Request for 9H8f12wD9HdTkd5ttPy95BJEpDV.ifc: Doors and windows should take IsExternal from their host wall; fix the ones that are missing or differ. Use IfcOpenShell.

First a look at what the model holds.

```python
import ifcopenshell
import ifcopenshell.util.element

model = ifcopenshell.open("9H8f12wD9HdTkd5ttPy95BJEpDV.ifc")
print(model.schema)
seen = {}
for e in model.by_type("IfcDoor") + model.by_type("IfcWindow"):
    if not e.FillsVoids:
        continue
    host = e.FillsVoids[0].RelatingOpeningElement.VoidsElements[0].RelatingBuildingElement
    own = ifcopenshell.util.element.get_pset(e, f"Pset_{e.is_a()[3:].removesuffix('StandardCase')}Common", "IsExternal")
    wall = ifcopenshell.util.element.get_pset(host, "Pset_WallCommon", "IsExternal")
    seen[e.is_a(), own, wall] = seen.get((e.is_a(), own, wall), 0) + 1
for (cls, own, wall), count in sorted(seen.items(), key=str):
    print(count, cls, "IsExternal:", own, "| host wall:", wall)
```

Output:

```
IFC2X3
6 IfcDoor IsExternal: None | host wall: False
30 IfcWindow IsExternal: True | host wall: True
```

```python
import ifcopenshell
import ifcopenshell.api.pset
import ifcopenshell.util.element

model = ifcopenshell.open("9H8f12wD9HdTkd5ttPy95BJEpDV.ifc")

count = 0
for ifc_class, pset_name in (("IfcDoor", "Pset_DoorCommon"), ("IfcWindow", "Pset_WindowCommon")):
    for e in model.by_type(ifc_class):
        if not e.FillsVoids:
            continue
        host = e.FillsVoids[0].RelatingOpeningElement.VoidsElements[0].RelatingBuildingElement
        external = ifcopenshell.util.element.get_pset(host, "Pset_WallCommon", "IsExternal")
        if external is None or ifcopenshell.util.element.get_pset(e, pset_name, "IsExternal") == external:
            continue
        pset = ifcopenshell.api.pset.add_pset(model, product=e, name=pset_name)
        ifcopenshell.api.pset.edit_pset(model, pset=pset, properties={"IsExternal": external})
        count += 1

print(count, "updated")

model.write("9H8f12wD9HdTkd5ttPy95BJEpDV-out.ifc")
```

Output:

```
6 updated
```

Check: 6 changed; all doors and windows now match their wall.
